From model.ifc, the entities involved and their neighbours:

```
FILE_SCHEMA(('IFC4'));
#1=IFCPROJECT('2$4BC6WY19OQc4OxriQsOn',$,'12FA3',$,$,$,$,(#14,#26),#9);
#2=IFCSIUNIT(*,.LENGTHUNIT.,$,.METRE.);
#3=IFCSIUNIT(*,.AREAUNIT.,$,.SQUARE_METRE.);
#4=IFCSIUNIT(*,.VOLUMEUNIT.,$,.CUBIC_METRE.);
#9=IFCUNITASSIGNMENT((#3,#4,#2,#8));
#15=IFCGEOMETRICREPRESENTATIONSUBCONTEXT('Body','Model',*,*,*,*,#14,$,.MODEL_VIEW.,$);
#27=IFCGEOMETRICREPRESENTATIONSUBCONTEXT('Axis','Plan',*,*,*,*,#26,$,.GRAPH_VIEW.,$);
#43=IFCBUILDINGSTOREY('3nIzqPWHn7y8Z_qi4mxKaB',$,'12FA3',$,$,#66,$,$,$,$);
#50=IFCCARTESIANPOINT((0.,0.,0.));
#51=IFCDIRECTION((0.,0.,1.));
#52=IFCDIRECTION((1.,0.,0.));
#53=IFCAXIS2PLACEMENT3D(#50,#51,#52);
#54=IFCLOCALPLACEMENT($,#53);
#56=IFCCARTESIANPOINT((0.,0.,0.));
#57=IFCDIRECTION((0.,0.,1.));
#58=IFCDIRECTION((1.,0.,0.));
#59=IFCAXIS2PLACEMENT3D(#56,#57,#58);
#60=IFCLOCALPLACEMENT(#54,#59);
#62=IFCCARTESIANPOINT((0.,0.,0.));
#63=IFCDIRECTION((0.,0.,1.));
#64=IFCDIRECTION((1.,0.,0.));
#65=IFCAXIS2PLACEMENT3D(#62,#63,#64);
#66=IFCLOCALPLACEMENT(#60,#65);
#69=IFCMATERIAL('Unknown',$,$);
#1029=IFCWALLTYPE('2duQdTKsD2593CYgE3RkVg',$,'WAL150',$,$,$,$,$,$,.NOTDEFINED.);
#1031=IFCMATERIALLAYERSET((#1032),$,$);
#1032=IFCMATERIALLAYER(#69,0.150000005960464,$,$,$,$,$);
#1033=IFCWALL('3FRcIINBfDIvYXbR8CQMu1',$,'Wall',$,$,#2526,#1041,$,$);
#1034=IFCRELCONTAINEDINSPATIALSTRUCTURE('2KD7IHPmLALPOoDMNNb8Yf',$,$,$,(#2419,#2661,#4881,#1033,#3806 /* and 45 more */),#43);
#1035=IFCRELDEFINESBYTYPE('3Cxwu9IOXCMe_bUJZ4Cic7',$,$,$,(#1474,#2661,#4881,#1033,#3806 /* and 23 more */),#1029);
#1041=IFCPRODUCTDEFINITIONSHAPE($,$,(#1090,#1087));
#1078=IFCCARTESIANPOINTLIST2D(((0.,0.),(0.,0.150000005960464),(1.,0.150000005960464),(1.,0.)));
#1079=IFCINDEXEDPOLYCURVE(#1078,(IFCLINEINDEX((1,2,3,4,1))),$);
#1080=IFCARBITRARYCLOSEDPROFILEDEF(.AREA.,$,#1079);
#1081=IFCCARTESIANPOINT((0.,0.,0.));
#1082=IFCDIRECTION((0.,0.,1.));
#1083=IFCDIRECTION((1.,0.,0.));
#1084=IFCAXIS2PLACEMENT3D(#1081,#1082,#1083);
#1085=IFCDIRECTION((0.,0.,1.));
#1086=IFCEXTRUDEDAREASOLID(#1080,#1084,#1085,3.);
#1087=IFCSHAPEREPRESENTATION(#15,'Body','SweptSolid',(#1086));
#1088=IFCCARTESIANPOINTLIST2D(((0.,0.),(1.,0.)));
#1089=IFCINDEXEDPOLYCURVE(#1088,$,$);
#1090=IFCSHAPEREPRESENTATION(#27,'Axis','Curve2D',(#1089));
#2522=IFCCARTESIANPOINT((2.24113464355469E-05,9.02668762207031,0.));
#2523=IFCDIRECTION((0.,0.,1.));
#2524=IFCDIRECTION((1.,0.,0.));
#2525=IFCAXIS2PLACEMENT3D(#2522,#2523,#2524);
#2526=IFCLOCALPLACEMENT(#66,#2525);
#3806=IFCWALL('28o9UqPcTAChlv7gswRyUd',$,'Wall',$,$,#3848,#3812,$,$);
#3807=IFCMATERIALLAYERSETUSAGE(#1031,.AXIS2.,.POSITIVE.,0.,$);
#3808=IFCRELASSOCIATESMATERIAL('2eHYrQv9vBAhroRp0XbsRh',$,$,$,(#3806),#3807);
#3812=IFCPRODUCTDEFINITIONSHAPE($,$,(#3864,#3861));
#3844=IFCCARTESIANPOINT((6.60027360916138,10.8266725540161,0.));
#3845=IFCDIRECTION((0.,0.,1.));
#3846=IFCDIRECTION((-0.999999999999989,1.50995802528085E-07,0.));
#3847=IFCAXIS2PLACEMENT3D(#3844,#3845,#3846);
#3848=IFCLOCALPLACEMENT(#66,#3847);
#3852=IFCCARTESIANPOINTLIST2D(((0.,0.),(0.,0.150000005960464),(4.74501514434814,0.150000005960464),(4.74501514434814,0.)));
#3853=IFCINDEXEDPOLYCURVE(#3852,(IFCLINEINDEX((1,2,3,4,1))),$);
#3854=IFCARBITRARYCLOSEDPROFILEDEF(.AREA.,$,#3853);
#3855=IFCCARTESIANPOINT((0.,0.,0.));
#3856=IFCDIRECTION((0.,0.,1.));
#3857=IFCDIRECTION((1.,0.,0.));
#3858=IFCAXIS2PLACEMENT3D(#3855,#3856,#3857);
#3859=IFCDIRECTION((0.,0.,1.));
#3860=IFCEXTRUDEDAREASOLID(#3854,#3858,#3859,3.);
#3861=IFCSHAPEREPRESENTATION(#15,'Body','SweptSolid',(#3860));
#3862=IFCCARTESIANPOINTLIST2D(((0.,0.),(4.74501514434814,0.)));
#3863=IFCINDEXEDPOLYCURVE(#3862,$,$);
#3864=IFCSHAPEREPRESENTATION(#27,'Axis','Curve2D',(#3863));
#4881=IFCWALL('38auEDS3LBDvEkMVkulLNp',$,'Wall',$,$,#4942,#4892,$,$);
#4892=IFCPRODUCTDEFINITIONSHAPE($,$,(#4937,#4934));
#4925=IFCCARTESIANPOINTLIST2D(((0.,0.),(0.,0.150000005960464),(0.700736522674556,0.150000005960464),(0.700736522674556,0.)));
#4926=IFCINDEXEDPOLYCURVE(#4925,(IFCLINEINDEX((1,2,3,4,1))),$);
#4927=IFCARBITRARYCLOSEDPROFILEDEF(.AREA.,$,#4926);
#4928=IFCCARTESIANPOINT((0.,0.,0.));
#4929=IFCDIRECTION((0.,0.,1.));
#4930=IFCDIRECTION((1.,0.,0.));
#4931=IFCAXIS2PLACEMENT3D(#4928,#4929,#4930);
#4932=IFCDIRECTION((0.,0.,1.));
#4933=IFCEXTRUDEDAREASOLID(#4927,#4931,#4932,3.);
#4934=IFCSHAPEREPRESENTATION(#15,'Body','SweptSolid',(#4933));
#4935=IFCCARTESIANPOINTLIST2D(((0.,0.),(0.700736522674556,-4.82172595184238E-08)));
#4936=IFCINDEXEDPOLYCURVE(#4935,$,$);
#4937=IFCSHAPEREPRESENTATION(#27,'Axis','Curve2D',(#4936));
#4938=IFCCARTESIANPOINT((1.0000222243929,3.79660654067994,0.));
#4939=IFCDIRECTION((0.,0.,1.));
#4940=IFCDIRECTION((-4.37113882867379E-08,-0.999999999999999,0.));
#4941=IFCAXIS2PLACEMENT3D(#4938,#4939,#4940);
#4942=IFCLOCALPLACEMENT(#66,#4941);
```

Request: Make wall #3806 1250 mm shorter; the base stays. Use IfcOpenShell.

```python
import ifcopenshell
import ifcopenshell.geom
import ifcopenshell.util.representation
import ifcopenshell.util.shape

model = ifcopenshell.open("model.ifc")
settings = ifcopenshell.geom.settings()


def volume(element):
    """Net volume in cubic metres, openings subtracted."""
    shape = ifcopenshell.geom.create_shape(settings, element)
    return ifcopenshell.util.shape.get_volume(shape.geometry)


wall = model.by_guid("28o9UqPcTAChlv7gswRyUd")
before = volume(wall)

body = ifcopenshell.util.representation.get_representation(wall, "Model", "Body")
solid = body.Items[0]
old_height = solid.Depth
solid.Depth -= 1.25
after = volume(wall)

print(f"height {old_height:g} -> {solid.Depth:g}, volume {before:.3f} -> {after:.3f} m3")

model.write("model_rev.ifc")
```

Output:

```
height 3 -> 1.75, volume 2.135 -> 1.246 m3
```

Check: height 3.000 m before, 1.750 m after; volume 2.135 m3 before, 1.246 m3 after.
